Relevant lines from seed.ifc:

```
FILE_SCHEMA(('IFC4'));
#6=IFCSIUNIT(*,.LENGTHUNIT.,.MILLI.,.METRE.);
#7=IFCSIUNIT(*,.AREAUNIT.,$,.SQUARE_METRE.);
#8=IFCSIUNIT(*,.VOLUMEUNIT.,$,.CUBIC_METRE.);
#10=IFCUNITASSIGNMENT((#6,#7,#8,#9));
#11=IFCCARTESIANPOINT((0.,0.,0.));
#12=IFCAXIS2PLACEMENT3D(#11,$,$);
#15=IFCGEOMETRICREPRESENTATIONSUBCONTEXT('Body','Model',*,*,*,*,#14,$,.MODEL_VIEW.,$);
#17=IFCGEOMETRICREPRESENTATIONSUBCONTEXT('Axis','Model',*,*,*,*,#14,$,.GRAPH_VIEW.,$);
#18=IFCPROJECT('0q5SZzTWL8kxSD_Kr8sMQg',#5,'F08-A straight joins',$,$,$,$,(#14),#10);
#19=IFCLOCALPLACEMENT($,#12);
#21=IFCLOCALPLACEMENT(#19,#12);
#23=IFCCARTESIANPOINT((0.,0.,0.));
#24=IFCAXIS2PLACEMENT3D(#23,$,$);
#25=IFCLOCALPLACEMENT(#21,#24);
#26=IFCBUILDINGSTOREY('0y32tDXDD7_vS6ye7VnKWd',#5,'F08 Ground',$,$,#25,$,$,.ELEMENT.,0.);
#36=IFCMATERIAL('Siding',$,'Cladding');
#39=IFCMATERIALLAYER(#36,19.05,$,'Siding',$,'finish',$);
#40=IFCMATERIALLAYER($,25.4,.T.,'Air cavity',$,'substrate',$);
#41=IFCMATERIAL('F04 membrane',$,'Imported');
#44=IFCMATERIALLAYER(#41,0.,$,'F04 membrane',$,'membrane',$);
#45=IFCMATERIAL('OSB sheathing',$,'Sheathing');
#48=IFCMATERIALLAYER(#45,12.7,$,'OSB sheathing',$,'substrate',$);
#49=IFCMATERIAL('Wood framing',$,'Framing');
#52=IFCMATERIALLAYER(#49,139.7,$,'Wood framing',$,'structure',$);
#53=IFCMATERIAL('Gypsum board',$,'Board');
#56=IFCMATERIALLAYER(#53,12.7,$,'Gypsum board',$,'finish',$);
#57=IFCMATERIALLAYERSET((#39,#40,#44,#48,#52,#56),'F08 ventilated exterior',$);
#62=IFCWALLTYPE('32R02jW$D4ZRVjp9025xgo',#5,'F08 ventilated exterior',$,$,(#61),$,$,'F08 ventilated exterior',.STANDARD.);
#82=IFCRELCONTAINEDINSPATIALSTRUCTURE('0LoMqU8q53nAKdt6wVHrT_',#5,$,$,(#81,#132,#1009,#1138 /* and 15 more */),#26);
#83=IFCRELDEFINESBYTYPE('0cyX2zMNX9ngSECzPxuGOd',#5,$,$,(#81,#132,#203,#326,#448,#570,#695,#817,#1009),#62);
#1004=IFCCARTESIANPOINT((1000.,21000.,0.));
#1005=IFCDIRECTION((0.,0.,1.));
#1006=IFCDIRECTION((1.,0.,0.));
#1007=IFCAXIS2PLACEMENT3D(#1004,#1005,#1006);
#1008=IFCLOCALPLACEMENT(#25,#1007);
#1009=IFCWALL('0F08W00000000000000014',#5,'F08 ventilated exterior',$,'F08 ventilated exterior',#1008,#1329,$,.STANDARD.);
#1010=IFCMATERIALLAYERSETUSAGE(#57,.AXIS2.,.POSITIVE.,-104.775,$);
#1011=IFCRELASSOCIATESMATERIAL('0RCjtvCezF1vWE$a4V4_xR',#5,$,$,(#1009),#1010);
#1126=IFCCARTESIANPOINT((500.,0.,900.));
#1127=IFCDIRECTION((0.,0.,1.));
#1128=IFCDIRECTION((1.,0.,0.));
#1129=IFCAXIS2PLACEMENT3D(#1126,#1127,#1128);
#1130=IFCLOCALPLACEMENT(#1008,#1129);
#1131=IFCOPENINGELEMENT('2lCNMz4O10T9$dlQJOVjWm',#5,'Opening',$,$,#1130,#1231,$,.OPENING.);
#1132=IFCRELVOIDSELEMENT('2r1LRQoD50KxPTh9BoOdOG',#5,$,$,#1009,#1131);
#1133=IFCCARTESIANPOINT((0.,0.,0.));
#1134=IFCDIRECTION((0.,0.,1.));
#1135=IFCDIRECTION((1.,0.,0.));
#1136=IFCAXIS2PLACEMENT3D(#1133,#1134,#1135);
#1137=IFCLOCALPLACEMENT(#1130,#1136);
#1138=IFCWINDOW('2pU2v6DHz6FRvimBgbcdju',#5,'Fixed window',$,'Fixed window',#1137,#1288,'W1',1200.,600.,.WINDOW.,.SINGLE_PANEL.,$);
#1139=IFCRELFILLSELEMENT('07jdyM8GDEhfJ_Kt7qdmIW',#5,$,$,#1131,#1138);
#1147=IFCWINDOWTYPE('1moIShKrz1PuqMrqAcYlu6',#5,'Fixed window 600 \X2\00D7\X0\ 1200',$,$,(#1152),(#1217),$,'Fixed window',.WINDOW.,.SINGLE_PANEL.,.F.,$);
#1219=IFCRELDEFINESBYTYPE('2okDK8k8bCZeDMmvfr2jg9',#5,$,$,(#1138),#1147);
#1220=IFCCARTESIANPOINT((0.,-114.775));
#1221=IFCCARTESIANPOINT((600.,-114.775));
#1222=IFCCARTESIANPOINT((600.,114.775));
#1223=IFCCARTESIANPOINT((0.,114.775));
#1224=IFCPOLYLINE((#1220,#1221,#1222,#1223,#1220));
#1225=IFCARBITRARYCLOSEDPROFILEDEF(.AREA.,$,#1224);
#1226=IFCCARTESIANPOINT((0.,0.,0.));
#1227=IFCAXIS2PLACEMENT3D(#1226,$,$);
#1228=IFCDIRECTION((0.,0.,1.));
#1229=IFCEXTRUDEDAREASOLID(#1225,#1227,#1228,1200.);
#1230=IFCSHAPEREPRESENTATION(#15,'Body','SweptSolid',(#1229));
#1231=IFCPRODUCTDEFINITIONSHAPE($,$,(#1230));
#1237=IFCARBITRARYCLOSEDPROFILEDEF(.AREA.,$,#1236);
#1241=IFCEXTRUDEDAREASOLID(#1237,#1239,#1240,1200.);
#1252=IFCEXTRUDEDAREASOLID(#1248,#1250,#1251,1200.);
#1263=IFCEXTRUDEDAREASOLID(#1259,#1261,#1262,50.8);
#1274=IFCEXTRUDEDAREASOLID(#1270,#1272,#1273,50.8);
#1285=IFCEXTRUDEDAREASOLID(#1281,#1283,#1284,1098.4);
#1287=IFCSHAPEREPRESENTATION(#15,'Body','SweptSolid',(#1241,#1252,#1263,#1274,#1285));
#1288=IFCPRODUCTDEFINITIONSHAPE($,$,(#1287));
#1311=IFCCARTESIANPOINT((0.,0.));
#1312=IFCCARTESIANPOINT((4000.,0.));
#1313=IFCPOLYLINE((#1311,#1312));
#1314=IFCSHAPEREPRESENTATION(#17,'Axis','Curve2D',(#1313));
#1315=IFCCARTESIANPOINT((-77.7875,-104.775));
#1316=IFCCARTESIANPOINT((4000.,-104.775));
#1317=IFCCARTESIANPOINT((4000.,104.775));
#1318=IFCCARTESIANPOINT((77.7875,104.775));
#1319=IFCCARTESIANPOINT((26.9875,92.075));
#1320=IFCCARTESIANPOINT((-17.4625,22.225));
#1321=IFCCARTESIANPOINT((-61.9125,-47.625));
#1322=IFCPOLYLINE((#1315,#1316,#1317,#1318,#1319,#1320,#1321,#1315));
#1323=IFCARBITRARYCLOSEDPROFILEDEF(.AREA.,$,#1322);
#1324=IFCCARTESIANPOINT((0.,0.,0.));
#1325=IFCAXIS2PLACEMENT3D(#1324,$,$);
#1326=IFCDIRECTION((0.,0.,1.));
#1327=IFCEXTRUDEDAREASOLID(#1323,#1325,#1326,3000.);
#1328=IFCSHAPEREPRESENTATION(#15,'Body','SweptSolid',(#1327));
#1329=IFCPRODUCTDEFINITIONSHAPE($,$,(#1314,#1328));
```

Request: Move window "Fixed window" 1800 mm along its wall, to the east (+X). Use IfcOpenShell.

```python
import ifcopenshell
import ifcopenshell.api.geometry
import ifcopenshell.util.placement
import ifcopenshell.util.unit

model = ifcopenshell.open("seed.ifc")
unit_scale = ifcopenshell.util.unit.calculate_unit_scale(model)

window = model.by_guid("2pU2v6DHz6FRvimBgbcdju")
opening = window.FillsVoids[0].RelatingOpeningElement
wall = opening.VoidsElements[0].RelatingBuildingElement

wall_matrix = ifcopenshell.util.placement.get_local_placement(wall.ObjectPlacement)
shift = wall_matrix[:3, 0] * 1.8 / unit_scale
before = ifcopenshell.util.placement.get_local_placement(window.ObjectPlacement)[:3, 3].copy()

# The window is placed relative to its opening, so it follows when the opening moves.
matrix = ifcopenshell.util.placement.get_local_placement(opening.ObjectPlacement)
matrix[:3, 3] += shift
ifcopenshell.api.geometry.edit_object_placement(
    model, product=opening, matrix=matrix, is_si=False, should_transform_children=True
)

after = ifcopenshell.util.placement.get_local_placement(window.ObjectPlacement)[:3, 3]
print("window moved by", (after - before).round(3) + 0.0)

model.write("seed_updated.ifc")
```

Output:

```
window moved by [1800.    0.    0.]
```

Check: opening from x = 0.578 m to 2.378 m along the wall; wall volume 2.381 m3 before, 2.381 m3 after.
